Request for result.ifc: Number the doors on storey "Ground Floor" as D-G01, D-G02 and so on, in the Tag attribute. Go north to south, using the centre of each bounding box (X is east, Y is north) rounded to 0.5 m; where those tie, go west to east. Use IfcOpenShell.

First a look at what the model holds.

```python
import ifcopenshell
import ifcopenshell.util.element
import ifcopenshell.util.placement

model = ifcopenshell.open("result.ifc")
print(model.schema)
storey = next(s for s in model.by_type("IfcBuildingStorey") if s.Name == "Ground Floor")
doors = [e for e in ifcopenshell.util.element.get_decomposition(storey) if e.is_a("IfcDoor")]
for e in sorted(doors, key=lambda e: e.id()):
    origin = ifcopenshell.util.placement.get_local_placement(e.ObjectPlacement)[:3, 3]
    print(e.id(), e.Tag, e.Name, origin.round(2) + 0.0, sep=" | ")
```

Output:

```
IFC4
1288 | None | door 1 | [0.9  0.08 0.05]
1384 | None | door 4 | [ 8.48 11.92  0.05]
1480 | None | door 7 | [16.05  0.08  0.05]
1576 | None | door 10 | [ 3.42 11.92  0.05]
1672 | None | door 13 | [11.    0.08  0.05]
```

```python
import ifcopenshell
import ifcopenshell.geom
import ifcopenshell.util.element
import ifcopenshell.util.shape

model = ifcopenshell.open("result.ifc")
settings = ifcopenshell.geom.settings()
settings.set("use-world-coords", True)


def centre(element):
    shape = ifcopenshell.geom.create_shape(settings, element)
    return ifcopenshell.util.shape.get_bbox_centroid(shape.geometry)


storey = next(s for s in model.by_type("IfcBuildingStorey") if s.Name == "Ground Floor")
doors = [e for e in ifcopenshell.util.element.get_decomposition(storey) if e.is_a("IfcDoor")]

# Insertion points can sit at a corner or the storey origin, so sort by the geometry (in metres).
centres = {e: centre(e) for e in doors}
doors.sort(key=lambda e: (-round(centres[e][1] / 0.5), centres[e][0]))

for i, e in enumerate(doors, start=1):
    number = f"D-G{i:02d}"
    e.Tag = number
    print(e.id(), number)

model.write("result_v2.ifc")
```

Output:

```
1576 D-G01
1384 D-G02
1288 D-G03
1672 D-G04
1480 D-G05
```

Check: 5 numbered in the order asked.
